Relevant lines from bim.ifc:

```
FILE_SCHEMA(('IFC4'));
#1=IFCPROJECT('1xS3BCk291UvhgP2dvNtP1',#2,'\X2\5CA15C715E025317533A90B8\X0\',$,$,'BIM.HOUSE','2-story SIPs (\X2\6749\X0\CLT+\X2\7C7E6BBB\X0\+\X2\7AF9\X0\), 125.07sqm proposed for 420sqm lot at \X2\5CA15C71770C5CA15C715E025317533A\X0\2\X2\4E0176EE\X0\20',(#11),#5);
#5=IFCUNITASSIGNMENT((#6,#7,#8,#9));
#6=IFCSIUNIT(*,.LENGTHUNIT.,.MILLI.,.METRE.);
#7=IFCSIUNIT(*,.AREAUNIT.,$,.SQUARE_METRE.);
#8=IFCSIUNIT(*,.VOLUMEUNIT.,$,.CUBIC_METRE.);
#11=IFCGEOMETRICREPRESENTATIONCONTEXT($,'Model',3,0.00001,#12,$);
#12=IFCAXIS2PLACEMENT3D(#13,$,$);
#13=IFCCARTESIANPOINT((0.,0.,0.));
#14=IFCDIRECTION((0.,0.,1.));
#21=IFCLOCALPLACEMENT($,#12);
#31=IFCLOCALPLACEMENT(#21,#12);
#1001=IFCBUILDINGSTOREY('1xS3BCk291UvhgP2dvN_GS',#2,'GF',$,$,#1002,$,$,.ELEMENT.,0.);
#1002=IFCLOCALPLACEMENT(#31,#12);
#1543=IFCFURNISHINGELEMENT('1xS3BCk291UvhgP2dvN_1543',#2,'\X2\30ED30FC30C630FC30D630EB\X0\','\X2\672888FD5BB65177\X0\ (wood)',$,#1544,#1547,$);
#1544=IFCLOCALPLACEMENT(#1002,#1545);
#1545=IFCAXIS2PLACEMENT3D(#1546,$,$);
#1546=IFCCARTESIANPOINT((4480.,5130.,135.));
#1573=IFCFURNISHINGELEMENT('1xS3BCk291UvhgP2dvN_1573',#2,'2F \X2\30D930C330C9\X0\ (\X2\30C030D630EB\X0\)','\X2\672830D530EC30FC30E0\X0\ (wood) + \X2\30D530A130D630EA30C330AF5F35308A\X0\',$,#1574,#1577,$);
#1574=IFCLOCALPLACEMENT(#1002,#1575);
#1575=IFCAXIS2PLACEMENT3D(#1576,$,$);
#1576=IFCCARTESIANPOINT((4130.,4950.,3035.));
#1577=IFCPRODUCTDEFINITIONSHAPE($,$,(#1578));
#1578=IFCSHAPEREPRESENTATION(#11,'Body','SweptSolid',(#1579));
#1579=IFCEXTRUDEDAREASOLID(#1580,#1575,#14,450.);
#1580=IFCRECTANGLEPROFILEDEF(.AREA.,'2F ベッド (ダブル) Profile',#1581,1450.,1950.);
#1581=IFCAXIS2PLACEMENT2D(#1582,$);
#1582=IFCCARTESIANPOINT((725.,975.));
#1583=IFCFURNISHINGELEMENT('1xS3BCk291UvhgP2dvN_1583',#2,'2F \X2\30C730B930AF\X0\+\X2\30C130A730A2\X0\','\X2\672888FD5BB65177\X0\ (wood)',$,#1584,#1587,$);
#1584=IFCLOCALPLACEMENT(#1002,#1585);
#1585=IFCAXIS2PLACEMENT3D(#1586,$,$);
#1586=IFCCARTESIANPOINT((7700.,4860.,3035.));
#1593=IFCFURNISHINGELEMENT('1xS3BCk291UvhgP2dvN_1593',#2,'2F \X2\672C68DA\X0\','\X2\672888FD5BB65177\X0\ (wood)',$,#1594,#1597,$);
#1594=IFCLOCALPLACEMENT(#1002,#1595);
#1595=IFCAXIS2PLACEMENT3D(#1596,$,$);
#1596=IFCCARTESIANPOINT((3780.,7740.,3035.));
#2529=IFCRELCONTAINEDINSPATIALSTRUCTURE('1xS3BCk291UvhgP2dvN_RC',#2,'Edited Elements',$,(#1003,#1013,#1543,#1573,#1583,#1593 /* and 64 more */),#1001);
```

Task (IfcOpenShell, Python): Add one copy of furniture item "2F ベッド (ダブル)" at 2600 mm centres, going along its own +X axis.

```python
import ifcopenshell
import ifcopenshell.api.geometry
import ifcopenshell.api.root
import ifcopenshell.util.element
import ifcopenshell.util.placement
import ifcopenshell.util.unit

model = ifcopenshell.open("bim.ifc")
unit_scale = ifcopenshell.util.unit.calculate_unit_scale(model)


def reuse_history(source, copy):
    """copy_class also copies each property set's owner history, people and application; keep the originals."""
    for rel in copy.IsDefinedBy:
        if rel.is_a("IfcRelDefinesByProperties") and (history := rel.RelatingPropertyDefinition.OwnerHistory):
            rel.RelatingPropertyDefinition.OwnerHistory = source.OwnerHistory
            ifcopenshell.util.element.remove_deep2(model, history)


source = model.by_guid("1xS3BCk291UvhgP2dvN_1573")
base = ifcopenshell.util.placement.get_local_placement(source.ObjectPlacement)
step = base[:3, 0] * 2.6 / unit_scale

for i in range(1, 2):
    copy = ifcopenshell.api.root.copy_class(model, product=source)
    copy.Representation = ifcopenshell.util.element.copy_deep(
        model, source.Representation, exclude=["IfcGeometricRepresentationContext", "IfcRepresentationMap"]
    )
    reuse_history(source, copy)
    matrix = base.copy()
    matrix[:3, 3] += i * step
    print("added at", matrix[:3, 3].round(3) + 0.0)
    ifcopenshell.api.geometry.edit_object_placement(model, product=copy, matrix=matrix, is_si=False)

model.write("bim_edited.ifc")
```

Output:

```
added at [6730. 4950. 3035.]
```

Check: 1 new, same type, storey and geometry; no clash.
